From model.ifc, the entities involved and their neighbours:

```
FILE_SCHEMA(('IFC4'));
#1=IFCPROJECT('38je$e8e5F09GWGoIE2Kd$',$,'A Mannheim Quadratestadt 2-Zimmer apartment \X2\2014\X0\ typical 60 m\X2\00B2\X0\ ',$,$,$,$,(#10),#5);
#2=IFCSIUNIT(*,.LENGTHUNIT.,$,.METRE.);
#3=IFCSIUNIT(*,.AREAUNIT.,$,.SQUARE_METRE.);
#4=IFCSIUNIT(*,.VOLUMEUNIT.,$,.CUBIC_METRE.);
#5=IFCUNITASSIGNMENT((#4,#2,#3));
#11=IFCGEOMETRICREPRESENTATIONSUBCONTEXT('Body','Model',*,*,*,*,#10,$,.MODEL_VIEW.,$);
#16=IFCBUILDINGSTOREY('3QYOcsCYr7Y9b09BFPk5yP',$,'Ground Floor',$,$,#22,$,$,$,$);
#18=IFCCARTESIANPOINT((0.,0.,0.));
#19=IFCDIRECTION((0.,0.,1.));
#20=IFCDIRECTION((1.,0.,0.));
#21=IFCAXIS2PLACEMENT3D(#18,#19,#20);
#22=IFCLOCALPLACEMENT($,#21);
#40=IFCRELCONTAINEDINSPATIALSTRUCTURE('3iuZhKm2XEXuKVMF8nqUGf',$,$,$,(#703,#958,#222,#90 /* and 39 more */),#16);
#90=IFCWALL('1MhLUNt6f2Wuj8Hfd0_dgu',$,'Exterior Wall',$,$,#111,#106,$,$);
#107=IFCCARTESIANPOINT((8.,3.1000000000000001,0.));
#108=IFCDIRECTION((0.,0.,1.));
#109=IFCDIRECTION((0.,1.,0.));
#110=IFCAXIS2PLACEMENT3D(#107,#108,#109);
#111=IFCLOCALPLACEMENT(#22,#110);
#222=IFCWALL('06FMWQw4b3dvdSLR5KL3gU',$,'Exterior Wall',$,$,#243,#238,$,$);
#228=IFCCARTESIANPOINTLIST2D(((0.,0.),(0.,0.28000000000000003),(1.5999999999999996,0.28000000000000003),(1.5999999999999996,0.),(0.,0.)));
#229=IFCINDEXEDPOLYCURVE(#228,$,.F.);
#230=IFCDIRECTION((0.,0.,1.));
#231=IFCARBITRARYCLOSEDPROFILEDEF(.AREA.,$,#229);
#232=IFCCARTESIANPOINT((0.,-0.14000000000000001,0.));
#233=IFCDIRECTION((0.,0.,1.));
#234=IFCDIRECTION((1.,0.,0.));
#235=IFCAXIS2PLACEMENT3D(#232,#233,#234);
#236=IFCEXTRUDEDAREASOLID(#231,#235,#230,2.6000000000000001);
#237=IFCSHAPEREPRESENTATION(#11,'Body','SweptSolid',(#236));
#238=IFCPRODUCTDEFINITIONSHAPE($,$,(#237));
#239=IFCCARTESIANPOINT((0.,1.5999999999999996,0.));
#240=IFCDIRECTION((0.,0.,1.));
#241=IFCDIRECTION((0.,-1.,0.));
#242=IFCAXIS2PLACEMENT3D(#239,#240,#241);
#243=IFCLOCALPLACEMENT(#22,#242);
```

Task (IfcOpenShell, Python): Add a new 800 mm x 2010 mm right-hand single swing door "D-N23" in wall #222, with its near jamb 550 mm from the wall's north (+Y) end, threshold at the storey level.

```python
import numpy as np
import ifcopenshell
import ifcopenshell.api.feature
import ifcopenshell.api.geometry
import ifcopenshell.api.root
import ifcopenshell.api.spatial
import ifcopenshell.geom
import ifcopenshell.util.element
import ifcopenshell.util.placement
import ifcopenshell.util.representation
import ifcopenshell.util.shape
import ifcopenshell.util.unit

model = ifcopenshell.open("model.ifc")
unit_scale = ifcopenshell.util.unit.calculate_unit_scale(model)
settings = ifcopenshell.geom.settings()


def volume(element):
    """Net volume in cubic metres, openings subtracted."""
    shape = ifcopenshell.geom.create_shape(settings, element)
    return ifcopenshell.util.shape.get_volume(shape.geometry)


wall = model.by_guid("06FMWQw4b3dvdSLR5KL3gU")
storey = ifcopenshell.util.element.get_container(wall, ifc_class="IfcBuildingStorey")
context = ifcopenshell.util.representation.get_context(model, "Model", "Body", "MODEL_VIEW")
before = volume(wall)

width, height, from_end, sill = 0.8, 2.01, 0.55, 0.0  # metres

# The wall runs along its own X axis, and the end named is its -X end.
wall_shape = ifcopenshell.geom.create_shape(settings, wall)
x, y, z = ifcopenshell.util.shape.get_vertices(wall_shape.geometry).T
start = x.min() + from_end
face, thickness = float(y.min()), float(y.max() - y.min())
wall_matrix = ifcopenshell.util.placement.get_local_placement(wall.ObjectPlacement)
level = ifcopenshell.util.placement.get_local_placement(storey.ObjectPlacement)[2, 3]


def in_wall(x, y):
    """Placement at x, y metres in the wall's axes, at sill height."""
    matrix = wall_matrix.copy()
    matrix[:, 3] = wall_matrix @ np.array([x / unit_scale, y / unit_scale, 0.0, 1.0])
    matrix[2, 3] = level + sill / unit_scale
    return matrix


# Opening: a box that overshoots both wall faces by 50 mm.
opening = ifcopenshell.api.root.create_entity(model, ifc_class="IfcOpeningElement", predefined_type="OPENING")
box = ifcopenshell.api.geometry.add_wall_representation(
    model, context=context, length=width, height=height, thickness=thickness + 0.1
)
ifcopenshell.api.geometry.assign_representation(model, product=opening, representation=box)
ifcopenshell.api.geometry.edit_object_placement(model, product=opening, matrix=in_wall(start, face - 0.05), is_si=False)
ifcopenshell.api.feature.add_feature(model, feature=opening, element=wall)

door = ifcopenshell.api.root.create_entity(model, ifc_class="IfcDoor", name="D-N23", predefined_type="DOOR")
door.OverallWidth, door.OverallHeight = width / unit_scale, height / unit_scale
door.OperationType = "SINGLE_SWING_RIGHT"
body = ifcopenshell.api.geometry.add_door_representation(
    model,
    context=context,
    overall_width=door.OverallWidth,
    overall_height=door.OverallHeight,
    operation_type="SINGLE_SWING_RIGHT",
    lining_properties={"LiningDepth": thickness / unit_scale, "ThresholdDepth": thickness / unit_scale},
)
ifcopenshell.api.geometry.assign_representation(model, product=door, representation=body)
ifcopenshell.api.spatial.assign_container(model, products=[door], relating_structure=storey)
ifcopenshell.api.feature.add_filling(model, opening=opening, element=door)

# The lining spans the wall, so the door starts at the wall face.
ifcopenshell.api.geometry.edit_object_placement(model, product=door, matrix=in_wall(start, face), is_si=False)

after = volume(wall)

print(f"wall volume {before:.3f} -> {after:.3f} m3")

model.write("model_updated.ifc")
```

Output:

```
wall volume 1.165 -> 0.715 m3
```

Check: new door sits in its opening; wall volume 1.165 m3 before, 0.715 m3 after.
